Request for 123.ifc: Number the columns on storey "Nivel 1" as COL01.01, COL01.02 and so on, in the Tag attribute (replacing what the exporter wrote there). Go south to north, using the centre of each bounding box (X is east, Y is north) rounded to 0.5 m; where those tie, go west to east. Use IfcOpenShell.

First a look at what the model holds.

```python
import ifcopenshell
import ifcopenshell.util.element
import ifcopenshell.util.placement

model = ifcopenshell.open("123.ifc")
print(model.schema)
storey = next(s for s in model.by_type("IfcBuildingStorey") if s.Name == "Nivel 1")
columns = [e for e in ifcopenshell.util.element.get_decomposition(storey) if e.is_a("IfcColumn")]
for e in sorted(columns, key=lambda e: e.id()):
    origin = ifcopenshell.util.placement.get_local_placement(e.ObjectPlacement)[:3, 3]
    print(e.id(), e.Tag, e.Name, origin.round(2) + 0.0, sep=" | ")
```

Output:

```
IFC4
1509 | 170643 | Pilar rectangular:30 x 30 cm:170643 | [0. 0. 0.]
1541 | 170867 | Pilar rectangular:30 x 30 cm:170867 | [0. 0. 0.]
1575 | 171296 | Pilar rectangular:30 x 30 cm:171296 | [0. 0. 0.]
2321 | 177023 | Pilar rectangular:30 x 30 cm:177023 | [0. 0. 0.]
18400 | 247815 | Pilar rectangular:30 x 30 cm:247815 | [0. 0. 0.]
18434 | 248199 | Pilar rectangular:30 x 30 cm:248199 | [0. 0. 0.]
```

```python
import ifcopenshell
import ifcopenshell.geom
import ifcopenshell.util.element
import ifcopenshell.util.shape

model = ifcopenshell.open("123.ifc")
settings = ifcopenshell.geom.settings()
settings.set("use-world-coords", True)


def centre(element):
    shape = ifcopenshell.geom.create_shape(settings, element)
    return ifcopenshell.util.shape.get_bbox_centroid(shape.geometry)


storey = next(s for s in model.by_type("IfcBuildingStorey") if s.Name == "Nivel 1")
columns = [e for e in ifcopenshell.util.element.get_decomposition(storey) if e.is_a("IfcColumn")]

# Insertion points can sit at a corner or the storey origin, so sort by the geometry (in metres).
centres = {e: centre(e) for e in columns}
columns.sort(key=lambda e: (round(centres[e][1] / 0.5), centres[e][0]))

for i, e in enumerate(columns, start=1):
    number = f"COL01.{i:02d}"
    e.Tag = number
    print(e.id(), number)

model.write("123_updated.ifc")
```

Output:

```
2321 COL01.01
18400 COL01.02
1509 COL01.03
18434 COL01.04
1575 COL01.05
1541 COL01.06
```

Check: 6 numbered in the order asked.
